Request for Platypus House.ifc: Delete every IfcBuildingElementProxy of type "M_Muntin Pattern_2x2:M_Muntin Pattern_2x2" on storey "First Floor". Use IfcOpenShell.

First a look at what the model holds.

```python
import ifcopenshell
import ifcopenshell.util.element

model = ifcopenshell.open("Platypus House.ifc")
print(model.schema)
storey = next(s for s in model.by_type("IfcBuildingStorey") if s.Name == "First Floor")
proxies = [e for e in ifcopenshell.util.element.get_decomposition(storey) if e.is_a("IfcBuildingElementProxy")]
seen = {}
for e in proxies:
    element_type = ifcopenshell.util.element.get_type(e)
    name = element_type.Name if element_type not in (None, e) else None
    seen[name] = seen.get(name, 0) + 1
for name, count in sorted(seen.items(), key=str):
    print(count, "x", name)
```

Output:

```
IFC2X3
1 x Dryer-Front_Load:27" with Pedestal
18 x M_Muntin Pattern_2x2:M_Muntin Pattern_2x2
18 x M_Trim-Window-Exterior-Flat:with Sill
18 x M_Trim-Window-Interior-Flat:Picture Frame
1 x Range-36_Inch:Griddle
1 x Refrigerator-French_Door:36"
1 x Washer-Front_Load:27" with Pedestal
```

```python
import ifcopenshell
import ifcopenshell.api.root
import ifcopenshell.util.element

model = ifcopenshell.open("Platypus House.ifc")

storey = next(s for s in model.by_type("IfcBuildingStorey") if s.Name == "First Floor")
proxies = [e for e in ifcopenshell.util.element.get_decomposition(storey) if e.is_a("IfcBuildingElementProxy")]
targets = [e for e in proxies if (t := ifcopenshell.util.element.get_type(e)) not in (None, e) and t.Name == "M_Muntin Pattern_2x2:M_Muntin Pattern_2x2"]

for e in targets:
    ifcopenshell.api.root.remove_product(model, product=e)
print(len(targets), "removed")

model.write("Platypus House_updated.ifc")
```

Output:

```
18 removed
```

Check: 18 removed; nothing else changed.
